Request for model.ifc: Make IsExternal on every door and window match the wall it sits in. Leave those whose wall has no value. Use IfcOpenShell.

First a look at what the model holds.

```python
import ifcopenshell
import ifcopenshell.util.element

model = ifcopenshell.open("model.ifc")
print(model.schema)
seen = {}
for e in model.by_type("IfcDoor") + model.by_type("IfcWindow"):
    if not e.FillsVoids:
        continue
    host = e.FillsVoids[0].RelatingOpeningElement.VoidsElements[0].RelatingBuildingElement
    own = ifcopenshell.util.element.get_pset(e, f"Pset_{e.is_a()[3:].removesuffix('StandardCase')}Common", "IsExternal")
    wall = ifcopenshell.util.element.get_pset(host, "Pset_WallCommon", "IsExternal")
    seen[e.is_a(), own, wall] = seen.get((e.is_a(), own, wall), 0) + 1
for (cls, own, wall), count in sorted(seen.items(), key=str):
    print(count, cls, "IsExternal:", own, "| host wall:", wall)
```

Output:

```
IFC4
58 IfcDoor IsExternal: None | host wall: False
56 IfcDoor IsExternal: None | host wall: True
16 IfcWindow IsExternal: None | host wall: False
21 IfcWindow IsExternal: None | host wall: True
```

```python
import ifcopenshell
import ifcopenshell.api.pset
import ifcopenshell.util.element

model = ifcopenshell.open("model.ifc")

count = 0
for ifc_class, pset_name in (("IfcDoor", "Pset_DoorCommon"), ("IfcWindow", "Pset_WindowCommon")):
    for e in model.by_type(ifc_class):
        if not e.FillsVoids:
            continue
        host = e.FillsVoids[0].RelatingOpeningElement.VoidsElements[0].RelatingBuildingElement
        external = ifcopenshell.util.element.get_pset(host, "Pset_WallCommon", "IsExternal")
        if external is None or ifcopenshell.util.element.get_pset(e, pset_name, "IsExternal") == external:
            continue
        pset = ifcopenshell.api.pset.add_pset(model, product=e, name=pset_name)
        ifcopenshell.api.pset.edit_pset(model, pset=pset, properties={"IsExternal": external})
        count += 1

print(count, "updated")

model.write("model_edited.ifc")
```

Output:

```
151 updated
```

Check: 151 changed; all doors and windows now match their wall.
